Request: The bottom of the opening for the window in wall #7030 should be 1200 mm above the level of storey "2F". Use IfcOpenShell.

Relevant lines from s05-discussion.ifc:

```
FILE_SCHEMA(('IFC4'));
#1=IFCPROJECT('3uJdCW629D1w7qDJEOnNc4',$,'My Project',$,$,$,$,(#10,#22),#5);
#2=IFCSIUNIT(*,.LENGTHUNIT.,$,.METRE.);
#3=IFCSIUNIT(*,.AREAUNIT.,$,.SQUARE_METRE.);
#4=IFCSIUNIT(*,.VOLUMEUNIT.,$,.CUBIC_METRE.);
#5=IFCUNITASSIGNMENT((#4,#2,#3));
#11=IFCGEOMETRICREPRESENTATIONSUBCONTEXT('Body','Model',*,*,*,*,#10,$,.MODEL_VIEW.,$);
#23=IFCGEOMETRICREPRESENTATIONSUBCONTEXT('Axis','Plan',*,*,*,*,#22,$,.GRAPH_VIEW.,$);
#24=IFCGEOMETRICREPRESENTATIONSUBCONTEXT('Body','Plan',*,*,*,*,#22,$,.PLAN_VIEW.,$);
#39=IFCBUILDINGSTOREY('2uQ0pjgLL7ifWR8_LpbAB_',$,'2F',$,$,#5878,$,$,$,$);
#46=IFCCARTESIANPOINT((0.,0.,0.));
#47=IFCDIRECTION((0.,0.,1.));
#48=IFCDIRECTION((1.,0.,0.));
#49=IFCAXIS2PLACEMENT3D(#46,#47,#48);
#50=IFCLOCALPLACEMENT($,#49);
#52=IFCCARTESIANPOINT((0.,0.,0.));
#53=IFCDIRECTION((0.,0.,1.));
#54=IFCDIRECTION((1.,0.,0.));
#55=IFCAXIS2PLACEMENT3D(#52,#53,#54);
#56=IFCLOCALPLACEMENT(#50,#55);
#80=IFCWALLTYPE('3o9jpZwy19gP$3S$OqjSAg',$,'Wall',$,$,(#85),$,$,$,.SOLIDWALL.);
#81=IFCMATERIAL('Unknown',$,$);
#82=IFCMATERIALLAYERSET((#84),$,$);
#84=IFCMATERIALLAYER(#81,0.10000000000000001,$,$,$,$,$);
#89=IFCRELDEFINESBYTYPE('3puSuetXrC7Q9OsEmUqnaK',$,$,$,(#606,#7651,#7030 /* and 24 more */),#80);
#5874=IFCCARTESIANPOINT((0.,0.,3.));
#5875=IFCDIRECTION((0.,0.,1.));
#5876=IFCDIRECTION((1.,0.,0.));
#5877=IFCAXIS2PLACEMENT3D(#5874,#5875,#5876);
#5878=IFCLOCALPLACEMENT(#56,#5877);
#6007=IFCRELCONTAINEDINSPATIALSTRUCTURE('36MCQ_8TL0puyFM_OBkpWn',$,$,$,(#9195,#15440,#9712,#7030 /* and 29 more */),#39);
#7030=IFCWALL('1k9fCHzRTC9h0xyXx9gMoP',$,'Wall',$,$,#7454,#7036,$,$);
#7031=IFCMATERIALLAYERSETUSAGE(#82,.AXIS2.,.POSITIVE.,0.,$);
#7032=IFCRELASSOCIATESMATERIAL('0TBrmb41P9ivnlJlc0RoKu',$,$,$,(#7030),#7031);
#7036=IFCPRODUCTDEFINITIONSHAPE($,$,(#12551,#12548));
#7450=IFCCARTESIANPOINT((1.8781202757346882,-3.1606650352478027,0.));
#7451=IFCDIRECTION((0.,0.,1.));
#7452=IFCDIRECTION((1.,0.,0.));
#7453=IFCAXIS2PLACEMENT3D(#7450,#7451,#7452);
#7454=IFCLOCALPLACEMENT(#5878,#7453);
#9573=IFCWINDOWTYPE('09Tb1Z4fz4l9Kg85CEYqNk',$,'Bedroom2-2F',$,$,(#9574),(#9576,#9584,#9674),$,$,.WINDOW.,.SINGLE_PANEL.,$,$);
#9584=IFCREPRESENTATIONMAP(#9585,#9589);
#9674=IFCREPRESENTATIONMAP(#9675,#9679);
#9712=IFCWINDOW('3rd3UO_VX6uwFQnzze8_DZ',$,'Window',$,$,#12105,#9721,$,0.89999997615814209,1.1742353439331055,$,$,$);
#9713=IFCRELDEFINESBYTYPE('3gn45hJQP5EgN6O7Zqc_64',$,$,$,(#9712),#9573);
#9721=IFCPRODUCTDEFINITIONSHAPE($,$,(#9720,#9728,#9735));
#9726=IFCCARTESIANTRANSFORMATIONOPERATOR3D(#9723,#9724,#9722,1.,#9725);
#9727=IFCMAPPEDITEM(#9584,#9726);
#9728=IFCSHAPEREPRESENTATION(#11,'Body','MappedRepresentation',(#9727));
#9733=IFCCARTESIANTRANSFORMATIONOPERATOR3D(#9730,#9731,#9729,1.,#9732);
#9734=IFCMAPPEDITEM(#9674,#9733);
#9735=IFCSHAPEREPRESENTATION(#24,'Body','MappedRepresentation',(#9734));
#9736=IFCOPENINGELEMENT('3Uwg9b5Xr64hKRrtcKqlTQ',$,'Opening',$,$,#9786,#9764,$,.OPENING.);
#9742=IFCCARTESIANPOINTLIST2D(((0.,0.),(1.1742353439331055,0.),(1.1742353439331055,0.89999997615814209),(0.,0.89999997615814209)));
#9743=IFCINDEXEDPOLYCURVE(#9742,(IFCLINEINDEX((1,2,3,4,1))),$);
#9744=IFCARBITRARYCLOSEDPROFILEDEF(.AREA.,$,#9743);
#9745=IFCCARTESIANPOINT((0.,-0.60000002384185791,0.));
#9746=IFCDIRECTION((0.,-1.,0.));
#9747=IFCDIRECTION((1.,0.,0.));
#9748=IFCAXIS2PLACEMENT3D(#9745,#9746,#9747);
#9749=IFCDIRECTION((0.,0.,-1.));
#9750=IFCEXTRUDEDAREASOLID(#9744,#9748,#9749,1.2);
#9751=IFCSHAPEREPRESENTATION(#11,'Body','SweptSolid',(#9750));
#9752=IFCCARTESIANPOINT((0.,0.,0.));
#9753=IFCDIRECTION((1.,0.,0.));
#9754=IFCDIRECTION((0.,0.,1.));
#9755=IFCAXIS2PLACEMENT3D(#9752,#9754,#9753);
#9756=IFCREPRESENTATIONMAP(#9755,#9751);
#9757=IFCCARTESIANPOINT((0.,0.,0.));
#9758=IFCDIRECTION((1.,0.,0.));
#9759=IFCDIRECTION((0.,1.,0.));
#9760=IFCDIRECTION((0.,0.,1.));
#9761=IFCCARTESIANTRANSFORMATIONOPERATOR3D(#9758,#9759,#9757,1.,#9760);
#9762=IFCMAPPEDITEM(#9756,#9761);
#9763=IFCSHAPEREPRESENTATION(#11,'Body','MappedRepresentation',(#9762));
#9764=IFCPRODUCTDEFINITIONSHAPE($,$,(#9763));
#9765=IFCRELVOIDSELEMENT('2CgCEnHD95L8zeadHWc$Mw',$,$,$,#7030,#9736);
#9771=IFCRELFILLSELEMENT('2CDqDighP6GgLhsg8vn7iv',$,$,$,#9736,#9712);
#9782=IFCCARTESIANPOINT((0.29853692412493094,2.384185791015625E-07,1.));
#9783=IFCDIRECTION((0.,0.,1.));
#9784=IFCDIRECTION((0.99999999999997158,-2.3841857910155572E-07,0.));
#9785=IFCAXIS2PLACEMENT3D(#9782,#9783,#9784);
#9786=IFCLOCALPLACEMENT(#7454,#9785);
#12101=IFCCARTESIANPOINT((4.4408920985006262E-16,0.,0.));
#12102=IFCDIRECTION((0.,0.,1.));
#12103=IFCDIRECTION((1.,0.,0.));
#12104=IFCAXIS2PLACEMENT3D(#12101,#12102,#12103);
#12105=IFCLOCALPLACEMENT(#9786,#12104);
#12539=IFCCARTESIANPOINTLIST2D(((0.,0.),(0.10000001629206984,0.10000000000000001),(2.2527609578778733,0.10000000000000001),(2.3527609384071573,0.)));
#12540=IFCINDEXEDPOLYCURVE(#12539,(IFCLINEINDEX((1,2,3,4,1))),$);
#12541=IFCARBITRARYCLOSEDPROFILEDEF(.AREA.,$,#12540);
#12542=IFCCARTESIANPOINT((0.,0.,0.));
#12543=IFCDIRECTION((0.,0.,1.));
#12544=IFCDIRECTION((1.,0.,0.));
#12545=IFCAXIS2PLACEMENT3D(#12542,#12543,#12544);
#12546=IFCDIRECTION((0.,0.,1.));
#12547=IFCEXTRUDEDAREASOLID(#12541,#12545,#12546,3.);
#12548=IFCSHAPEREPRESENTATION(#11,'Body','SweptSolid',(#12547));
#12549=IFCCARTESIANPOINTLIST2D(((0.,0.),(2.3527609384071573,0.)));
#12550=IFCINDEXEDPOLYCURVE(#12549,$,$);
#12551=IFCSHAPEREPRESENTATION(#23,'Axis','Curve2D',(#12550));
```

```python
import numpy as np
import ifcopenshell
import ifcopenshell.api.geometry
import ifcopenshell.geom
import ifcopenshell.util.element
import ifcopenshell.util.placement
import ifcopenshell.util.shape
import ifcopenshell.util.unit

model = ifcopenshell.open("s05-discussion.ifc")
unit_scale = ifcopenshell.util.unit.calculate_unit_scale(model)

window = model.by_guid("3rd3UO_VX6uwFQnzze8_DZ")
opening = window.FillsVoids[0].RelatingOpeningElement
storey = ifcopenshell.util.element.get_container(window, ifc_class="IfcBuildingStorey")
level = ifcopenshell.util.placement.get_local_placement(storey.ObjectPlacement)[2, 3]

# The opening's origin need not be at the sill, so measure its lowest point.
shape = ifcopenshell.geom.create_shape(ifcopenshell.geom.settings(), opening)
bottom = ifcopenshell.util.shape.get_shape_bottom_elevation(shape, shape.geometry) / unit_scale
dz = level + 1.2 / unit_scale - bottom

shift = np.array([0.0, 0.0, dz])
# The window is placed relative to its opening, so it follows when the opening moves.
matrix = ifcopenshell.util.placement.get_local_placement(opening.ObjectPlacement)
matrix[:3, 3] += shift
ifcopenshell.api.geometry.edit_object_placement(
    model, product=opening, matrix=matrix, is_si=False, should_transform_children=True
)

print(f"moved by {dz * unit_scale:+.3f} m")

model.write("s05-discussion_v2.ifc")
```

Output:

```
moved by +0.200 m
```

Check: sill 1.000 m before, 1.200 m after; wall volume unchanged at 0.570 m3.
